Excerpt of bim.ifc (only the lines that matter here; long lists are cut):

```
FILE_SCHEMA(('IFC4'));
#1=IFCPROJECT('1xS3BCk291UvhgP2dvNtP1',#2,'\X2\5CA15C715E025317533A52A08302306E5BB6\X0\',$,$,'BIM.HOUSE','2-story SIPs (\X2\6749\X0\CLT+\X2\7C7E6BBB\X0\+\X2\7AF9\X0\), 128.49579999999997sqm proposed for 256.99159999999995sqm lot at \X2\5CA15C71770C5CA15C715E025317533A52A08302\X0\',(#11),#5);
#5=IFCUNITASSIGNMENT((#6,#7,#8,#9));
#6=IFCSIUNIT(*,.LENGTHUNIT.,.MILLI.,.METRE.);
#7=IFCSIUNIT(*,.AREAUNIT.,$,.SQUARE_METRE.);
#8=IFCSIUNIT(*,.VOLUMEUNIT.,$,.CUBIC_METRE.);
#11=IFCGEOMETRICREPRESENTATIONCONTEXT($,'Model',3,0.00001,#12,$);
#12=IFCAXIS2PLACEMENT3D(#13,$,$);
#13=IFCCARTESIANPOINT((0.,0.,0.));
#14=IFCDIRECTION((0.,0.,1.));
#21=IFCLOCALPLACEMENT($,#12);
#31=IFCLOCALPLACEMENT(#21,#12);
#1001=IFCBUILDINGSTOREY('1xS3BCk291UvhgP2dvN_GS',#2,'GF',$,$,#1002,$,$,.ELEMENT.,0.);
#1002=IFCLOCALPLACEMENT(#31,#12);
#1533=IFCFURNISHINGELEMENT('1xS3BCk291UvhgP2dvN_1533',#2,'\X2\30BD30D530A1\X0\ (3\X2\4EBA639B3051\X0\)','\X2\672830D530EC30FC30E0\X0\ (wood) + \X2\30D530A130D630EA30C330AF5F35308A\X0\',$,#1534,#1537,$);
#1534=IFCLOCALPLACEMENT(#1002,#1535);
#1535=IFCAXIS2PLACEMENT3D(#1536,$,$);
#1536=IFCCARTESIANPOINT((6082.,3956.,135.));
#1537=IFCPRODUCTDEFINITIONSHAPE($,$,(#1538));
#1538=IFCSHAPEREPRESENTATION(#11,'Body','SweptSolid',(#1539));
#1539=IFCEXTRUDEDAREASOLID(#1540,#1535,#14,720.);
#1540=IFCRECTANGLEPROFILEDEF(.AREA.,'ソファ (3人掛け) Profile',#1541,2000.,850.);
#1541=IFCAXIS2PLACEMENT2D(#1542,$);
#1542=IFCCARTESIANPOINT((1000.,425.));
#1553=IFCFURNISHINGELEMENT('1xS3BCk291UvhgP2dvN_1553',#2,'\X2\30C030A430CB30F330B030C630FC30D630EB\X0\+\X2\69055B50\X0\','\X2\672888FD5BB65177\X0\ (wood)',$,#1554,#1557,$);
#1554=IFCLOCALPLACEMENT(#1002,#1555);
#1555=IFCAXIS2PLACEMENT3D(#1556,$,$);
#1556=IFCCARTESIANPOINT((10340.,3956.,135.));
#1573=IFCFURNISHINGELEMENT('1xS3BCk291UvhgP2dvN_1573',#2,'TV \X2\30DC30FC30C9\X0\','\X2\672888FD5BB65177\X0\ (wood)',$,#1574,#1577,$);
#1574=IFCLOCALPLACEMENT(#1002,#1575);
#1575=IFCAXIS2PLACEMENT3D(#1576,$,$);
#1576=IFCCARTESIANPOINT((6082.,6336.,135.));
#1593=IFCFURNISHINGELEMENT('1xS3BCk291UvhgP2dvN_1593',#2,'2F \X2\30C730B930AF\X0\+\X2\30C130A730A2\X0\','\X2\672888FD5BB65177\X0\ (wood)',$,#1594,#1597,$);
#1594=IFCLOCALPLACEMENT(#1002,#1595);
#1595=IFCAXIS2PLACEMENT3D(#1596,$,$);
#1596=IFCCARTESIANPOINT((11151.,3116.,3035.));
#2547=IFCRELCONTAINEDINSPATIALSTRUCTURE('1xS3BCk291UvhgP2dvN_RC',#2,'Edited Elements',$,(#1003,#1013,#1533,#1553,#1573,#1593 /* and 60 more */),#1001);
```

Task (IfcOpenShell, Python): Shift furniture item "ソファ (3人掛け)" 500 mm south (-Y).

```python
import ifcopenshell
import ifcopenshell.api.geometry
import ifcopenshell.util.placement
import ifcopenshell.util.unit

model = ifcopenshell.open("bim.ifc")
unit_scale = ifcopenshell.util.unit.calculate_unit_scale(model)

item = model.by_guid("1xS3BCk291UvhgP2dvN_1533")
matrix = ifcopenshell.util.placement.get_local_placement(item.ObjectPlacement)
matrix[1, 3] -= 0.5 / unit_scale
ifcopenshell.api.geometry.edit_object_placement(model, product=item, matrix=matrix, is_si=False)

print(ifcopenshell.util.placement.get_local_placement(item.ObjectPlacement).round(3) + 0.0)

model.write("bim-out.ifc")
```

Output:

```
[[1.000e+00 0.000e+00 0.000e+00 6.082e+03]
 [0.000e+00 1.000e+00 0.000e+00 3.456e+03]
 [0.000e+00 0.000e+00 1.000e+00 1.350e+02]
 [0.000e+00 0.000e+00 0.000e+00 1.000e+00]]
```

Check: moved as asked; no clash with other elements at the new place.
